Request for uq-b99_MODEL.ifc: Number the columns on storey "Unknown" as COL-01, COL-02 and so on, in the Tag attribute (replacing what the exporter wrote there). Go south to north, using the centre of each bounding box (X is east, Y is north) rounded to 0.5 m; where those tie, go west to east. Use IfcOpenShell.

First a look at what the model holds.

```python
import ifcopenshell
import ifcopenshell.util.element
import ifcopenshell.util.placement

model = ifcopenshell.open("uq-b99_MODEL.ifc")
print(model.schema)
storey = next(s for s in model.by_type("IfcBuildingStorey") if s.Name == "Unknown")
columns = [e for e in ifcopenshell.util.element.get_decomposition(storey) if e.is_a("IfcColumn")]
for e in sorted(columns, key=lambda e: e.id()):
    origin = ifcopenshell.util.placement.get_local_placement(e.ObjectPlacement)[:3, 3]
    print(e.id(), e.Tag, e.Name, origin.round(2) + 0.0, sep=" | ")
```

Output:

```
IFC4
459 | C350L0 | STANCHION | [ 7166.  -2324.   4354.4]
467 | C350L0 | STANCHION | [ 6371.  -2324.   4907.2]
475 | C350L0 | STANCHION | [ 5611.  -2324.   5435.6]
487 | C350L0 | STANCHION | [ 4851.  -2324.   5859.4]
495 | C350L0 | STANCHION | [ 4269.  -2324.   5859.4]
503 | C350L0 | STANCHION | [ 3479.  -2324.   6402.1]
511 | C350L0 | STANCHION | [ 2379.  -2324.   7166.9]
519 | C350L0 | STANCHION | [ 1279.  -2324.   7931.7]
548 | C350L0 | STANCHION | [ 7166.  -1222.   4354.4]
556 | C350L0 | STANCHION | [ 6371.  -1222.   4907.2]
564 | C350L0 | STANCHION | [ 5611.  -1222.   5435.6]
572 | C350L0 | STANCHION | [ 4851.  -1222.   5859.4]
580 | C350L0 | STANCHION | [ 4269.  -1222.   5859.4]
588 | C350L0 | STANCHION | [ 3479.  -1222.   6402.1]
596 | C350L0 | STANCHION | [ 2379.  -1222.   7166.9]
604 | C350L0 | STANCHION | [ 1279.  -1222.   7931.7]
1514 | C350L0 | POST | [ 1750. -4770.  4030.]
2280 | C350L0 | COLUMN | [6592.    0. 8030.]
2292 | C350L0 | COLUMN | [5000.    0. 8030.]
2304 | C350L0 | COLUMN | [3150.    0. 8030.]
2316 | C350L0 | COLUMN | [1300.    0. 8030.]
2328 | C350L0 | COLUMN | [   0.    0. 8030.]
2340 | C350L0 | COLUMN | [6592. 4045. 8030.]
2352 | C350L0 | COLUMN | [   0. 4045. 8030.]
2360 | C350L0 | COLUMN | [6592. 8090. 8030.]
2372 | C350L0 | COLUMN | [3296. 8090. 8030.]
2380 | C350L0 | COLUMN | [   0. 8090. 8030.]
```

```python
import ifcopenshell
import ifcopenshell.geom
import ifcopenshell.util.element
import ifcopenshell.util.shape

model = ifcopenshell.open("uq-b99_MODEL.ifc")
settings = ifcopenshell.geom.settings()
settings.set("use-world-coords", True)


def centre(element):
    shape = ifcopenshell.geom.create_shape(settings, element)
    return ifcopenshell.util.shape.get_bbox_centroid(shape.geometry)


storey = next(s for s in model.by_type("IfcBuildingStorey") if s.Name == "Unknown")
columns = [e for e in ifcopenshell.util.element.get_decomposition(storey) if e.is_a("IfcColumn")]

# Insertion points can sit at a corner or the storey origin, so sort by the geometry (in metres).
centres = {e: centre(e) for e in columns}
columns.sort(key=lambda e: (round(centres[e][1] / 0.5), centres[e][0]))

for i, e in enumerate(columns, start=1):
    number = f"COL-{i:02d}"
    e.Tag = number
    print(e.id(), number)

model.write("uq-b99_MODEL_rev.ifc")
```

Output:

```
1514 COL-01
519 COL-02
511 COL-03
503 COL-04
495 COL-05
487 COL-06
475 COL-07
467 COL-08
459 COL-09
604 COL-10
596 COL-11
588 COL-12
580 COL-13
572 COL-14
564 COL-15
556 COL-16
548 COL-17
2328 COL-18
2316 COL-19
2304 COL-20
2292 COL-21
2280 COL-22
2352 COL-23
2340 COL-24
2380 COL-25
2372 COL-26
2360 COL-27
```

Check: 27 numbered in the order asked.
